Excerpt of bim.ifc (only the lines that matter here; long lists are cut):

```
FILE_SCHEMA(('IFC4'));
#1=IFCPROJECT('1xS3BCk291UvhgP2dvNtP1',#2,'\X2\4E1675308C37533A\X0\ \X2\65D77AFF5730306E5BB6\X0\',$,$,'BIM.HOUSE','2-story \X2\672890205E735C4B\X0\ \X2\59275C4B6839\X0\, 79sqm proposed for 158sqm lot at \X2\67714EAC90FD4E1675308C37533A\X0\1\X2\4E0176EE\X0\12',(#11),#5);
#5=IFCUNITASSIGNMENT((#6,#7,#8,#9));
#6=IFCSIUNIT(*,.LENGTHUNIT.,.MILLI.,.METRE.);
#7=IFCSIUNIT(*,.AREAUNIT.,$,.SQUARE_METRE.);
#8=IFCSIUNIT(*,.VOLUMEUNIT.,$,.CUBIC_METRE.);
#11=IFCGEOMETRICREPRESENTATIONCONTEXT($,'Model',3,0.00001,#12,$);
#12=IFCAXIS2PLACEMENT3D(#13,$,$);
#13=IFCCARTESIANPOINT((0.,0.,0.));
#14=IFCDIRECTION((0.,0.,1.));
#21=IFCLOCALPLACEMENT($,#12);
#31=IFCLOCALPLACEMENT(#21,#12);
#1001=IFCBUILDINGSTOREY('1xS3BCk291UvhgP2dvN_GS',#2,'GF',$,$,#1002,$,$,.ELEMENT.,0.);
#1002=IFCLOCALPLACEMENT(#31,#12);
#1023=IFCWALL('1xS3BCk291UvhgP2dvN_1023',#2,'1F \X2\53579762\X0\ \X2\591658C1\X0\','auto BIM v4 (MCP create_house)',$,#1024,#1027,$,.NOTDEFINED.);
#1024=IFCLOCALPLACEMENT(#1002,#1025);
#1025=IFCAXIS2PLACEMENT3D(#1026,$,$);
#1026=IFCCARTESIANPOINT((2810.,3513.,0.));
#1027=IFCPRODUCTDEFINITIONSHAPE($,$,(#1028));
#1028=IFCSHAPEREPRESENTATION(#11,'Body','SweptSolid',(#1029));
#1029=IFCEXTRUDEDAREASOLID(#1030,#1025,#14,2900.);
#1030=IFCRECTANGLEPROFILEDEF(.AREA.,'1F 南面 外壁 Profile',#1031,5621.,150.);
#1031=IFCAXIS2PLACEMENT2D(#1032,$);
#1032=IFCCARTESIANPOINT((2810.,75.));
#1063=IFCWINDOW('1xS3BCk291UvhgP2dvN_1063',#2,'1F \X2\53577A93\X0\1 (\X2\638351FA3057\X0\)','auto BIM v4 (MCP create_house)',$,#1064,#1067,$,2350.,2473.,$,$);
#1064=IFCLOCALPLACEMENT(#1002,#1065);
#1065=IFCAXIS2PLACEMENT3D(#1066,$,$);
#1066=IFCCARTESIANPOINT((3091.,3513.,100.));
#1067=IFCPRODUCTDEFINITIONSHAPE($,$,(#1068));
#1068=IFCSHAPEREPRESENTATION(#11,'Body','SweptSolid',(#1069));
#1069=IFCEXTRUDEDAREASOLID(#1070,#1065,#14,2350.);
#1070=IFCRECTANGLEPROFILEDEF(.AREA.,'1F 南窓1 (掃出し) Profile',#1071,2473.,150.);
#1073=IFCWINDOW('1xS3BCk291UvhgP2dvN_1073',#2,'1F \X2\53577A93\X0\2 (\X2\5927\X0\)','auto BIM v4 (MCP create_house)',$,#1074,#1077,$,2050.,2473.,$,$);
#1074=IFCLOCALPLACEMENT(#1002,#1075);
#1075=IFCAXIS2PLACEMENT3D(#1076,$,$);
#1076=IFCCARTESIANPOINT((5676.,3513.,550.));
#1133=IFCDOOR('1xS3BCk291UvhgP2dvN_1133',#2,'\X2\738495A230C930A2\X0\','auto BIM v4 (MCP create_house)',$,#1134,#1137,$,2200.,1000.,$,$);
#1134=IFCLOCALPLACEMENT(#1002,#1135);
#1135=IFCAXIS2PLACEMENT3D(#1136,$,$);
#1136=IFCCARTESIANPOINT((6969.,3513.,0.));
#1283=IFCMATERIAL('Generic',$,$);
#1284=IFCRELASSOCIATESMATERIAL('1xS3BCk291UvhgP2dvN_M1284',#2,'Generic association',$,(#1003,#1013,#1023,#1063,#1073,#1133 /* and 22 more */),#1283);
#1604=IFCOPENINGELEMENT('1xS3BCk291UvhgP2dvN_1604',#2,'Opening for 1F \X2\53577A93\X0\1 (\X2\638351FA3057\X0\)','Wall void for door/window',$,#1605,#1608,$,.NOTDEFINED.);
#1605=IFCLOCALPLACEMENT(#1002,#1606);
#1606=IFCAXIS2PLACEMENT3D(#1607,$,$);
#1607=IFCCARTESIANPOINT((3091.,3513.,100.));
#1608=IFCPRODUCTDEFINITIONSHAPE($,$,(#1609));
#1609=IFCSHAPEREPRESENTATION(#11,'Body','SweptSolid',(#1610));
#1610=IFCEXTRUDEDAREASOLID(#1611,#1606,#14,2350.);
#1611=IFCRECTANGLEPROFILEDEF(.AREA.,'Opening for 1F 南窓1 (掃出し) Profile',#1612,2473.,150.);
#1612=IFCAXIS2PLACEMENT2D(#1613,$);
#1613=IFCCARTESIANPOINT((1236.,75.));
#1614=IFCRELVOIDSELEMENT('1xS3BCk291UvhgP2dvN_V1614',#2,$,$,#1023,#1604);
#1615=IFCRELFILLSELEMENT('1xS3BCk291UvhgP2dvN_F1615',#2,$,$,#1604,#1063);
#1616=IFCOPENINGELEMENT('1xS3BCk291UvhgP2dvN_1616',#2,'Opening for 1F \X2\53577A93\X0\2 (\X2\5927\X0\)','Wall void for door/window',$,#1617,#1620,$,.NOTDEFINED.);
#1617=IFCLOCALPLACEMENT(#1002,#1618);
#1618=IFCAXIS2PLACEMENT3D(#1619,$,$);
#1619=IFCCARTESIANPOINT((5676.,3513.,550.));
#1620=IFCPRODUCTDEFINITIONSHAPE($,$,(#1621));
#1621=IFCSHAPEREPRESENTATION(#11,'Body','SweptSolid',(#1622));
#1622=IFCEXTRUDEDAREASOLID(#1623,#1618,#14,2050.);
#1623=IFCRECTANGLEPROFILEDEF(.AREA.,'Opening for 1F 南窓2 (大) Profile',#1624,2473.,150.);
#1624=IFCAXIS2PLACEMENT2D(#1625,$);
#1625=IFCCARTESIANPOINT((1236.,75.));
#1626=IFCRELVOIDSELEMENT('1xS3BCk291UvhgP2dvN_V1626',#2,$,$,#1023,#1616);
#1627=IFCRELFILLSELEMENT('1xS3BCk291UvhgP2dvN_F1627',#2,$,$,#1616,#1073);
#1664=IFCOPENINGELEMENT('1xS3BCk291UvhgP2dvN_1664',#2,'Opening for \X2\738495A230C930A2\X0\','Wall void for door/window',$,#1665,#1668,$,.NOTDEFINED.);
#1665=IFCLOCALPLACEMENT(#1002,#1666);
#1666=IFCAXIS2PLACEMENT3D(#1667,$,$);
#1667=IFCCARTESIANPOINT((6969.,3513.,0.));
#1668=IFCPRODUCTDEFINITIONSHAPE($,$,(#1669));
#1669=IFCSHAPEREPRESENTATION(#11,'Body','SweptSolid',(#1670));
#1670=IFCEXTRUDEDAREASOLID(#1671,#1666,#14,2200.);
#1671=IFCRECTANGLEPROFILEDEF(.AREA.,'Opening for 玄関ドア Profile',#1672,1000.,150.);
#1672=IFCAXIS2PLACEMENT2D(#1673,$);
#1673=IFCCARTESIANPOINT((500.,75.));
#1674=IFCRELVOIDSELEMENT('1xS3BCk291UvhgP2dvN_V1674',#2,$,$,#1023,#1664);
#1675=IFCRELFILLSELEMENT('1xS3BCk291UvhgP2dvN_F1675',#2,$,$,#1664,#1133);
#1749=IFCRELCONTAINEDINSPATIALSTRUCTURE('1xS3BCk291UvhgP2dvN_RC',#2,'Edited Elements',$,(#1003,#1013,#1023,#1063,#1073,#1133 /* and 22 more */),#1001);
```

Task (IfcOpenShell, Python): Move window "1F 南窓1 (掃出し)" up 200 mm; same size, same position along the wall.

```python
import numpy as np
import ifcopenshell
import ifcopenshell.api.geometry
import ifcopenshell.util.placement
import ifcopenshell.util.unit

model = ifcopenshell.open("bim.ifc")
unit_scale = ifcopenshell.util.unit.calculate_unit_scale(model)

window = model.by_guid("1xS3BCk291UvhgP2dvN_1063")
opening = window.FillsVoids[0].RelatingOpeningElement
dz = 0.2 / unit_scale

shift = np.array([0.0, 0.0, dz])
# The window is not placed relative to its opening, so move both.
for product in (opening, window):
    matrix = ifcopenshell.util.placement.get_local_placement(product.ObjectPlacement)
    matrix[:3, 3] += shift
    ifcopenshell.api.geometry.edit_object_placement(model, product=product, matrix=matrix, is_si=False)

print(f"moved by {dz * unit_scale:+.3f} m")

model.write("bim-out.ifc")
```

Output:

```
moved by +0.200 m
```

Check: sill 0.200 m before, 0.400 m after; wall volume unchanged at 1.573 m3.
